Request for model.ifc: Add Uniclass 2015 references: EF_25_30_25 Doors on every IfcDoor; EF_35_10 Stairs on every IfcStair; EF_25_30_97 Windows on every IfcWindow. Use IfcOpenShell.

First a look at what the model holds.

```python
import ifcopenshell

model = ifcopenshell.open("model.ifc")
print(model.schema)
print("classifications:", [c.Name for c in model.by_type("IfcClassification")])
for ifc_class in ("IfcDoor", "IfcRoof", "IfcStair", "IfcWall", "IfcWindow"):
    print(ifc_class, len(model.by_type(ifc_class)))
```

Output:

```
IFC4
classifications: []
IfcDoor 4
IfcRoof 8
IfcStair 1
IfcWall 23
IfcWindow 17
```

```python
import ifcopenshell
import ifcopenshell.api.classification

model = ifcopenshell.open("model.ifc")

system = ifcopenshell.api.classification.add_classification(model, classification="Uniclass 2015")

codes = {
    "IfcDoor": ("EF_25_30_25", "Doors"),
    "IfcStair": ("EF_35_10", "Stairs"),
    "IfcWindow": ("EF_25_30_97", "Windows"),
}
for ifc_class, (code, name) in codes.items():
    products = model.by_type(ifc_class)
    ifcopenshell.api.classification.add_reference(
        model, products=products, classification=system, identification=code, name=name
    )
    print(code, len(products))

model.write("model_edited.ifc")
```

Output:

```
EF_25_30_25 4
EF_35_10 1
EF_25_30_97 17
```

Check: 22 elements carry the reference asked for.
